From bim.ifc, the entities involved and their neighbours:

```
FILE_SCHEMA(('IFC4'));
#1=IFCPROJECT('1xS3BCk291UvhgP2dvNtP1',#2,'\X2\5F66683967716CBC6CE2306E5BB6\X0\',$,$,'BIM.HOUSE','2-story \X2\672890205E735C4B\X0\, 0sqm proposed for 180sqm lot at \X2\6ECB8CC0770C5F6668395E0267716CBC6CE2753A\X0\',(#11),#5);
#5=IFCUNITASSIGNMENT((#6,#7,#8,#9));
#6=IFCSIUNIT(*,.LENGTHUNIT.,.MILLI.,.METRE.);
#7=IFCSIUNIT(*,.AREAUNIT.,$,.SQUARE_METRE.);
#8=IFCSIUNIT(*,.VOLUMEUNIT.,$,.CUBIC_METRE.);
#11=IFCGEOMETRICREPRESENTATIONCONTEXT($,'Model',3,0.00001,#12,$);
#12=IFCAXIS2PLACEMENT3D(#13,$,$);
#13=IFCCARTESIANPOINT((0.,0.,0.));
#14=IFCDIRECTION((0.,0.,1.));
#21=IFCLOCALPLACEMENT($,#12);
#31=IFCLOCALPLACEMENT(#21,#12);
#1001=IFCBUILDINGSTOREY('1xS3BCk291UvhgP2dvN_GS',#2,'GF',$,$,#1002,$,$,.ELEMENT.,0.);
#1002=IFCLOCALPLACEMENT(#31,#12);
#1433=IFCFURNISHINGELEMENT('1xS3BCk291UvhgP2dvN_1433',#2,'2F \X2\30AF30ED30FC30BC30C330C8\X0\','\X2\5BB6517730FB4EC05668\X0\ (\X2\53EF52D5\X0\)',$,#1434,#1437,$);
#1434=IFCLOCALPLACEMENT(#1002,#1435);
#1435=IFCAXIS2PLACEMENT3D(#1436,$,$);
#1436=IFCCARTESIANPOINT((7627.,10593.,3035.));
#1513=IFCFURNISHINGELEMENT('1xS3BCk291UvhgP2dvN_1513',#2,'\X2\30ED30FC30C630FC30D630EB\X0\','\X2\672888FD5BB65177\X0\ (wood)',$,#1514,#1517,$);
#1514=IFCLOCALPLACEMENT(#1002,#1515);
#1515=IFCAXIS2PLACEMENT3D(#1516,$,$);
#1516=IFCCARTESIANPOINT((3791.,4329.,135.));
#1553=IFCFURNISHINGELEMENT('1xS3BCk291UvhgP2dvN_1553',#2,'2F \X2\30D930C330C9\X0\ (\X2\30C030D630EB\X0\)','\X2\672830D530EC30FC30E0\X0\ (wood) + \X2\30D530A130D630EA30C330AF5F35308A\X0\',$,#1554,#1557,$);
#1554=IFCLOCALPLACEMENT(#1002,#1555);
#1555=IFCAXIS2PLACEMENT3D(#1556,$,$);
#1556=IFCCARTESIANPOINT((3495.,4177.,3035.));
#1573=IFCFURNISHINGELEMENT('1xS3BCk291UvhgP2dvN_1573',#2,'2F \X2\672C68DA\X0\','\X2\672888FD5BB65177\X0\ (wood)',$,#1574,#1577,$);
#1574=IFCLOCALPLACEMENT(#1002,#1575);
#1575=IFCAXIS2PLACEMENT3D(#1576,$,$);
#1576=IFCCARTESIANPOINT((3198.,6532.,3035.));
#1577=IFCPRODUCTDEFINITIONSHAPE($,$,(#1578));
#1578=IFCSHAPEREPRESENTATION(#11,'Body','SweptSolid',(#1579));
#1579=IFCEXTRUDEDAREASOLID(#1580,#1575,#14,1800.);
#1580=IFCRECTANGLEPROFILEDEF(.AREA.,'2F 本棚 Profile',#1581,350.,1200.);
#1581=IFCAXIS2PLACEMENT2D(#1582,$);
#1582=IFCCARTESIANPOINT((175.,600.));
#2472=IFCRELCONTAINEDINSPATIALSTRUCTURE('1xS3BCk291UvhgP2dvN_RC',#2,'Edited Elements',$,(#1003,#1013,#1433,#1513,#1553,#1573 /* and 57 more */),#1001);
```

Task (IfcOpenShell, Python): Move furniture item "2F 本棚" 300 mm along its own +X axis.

```python
import ifcopenshell
import ifcopenshell.api.geometry
import ifcopenshell.util.placement

model = ifcopenshell.open("bim.ifc")

item = model.by_id(1573)
matrix = ifcopenshell.util.placement.get_local_placement(item.ObjectPlacement)
matrix[:3, 3] += matrix[:3, 0] * 300.0
ifcopenshell.api.geometry.edit_object_placement(model, product=item, matrix=matrix, is_si=False)

print(ifcopenshell.util.placement.get_local_placement(item.ObjectPlacement).round(3) + 0.0)

model.write("bim_updated.ifc")
```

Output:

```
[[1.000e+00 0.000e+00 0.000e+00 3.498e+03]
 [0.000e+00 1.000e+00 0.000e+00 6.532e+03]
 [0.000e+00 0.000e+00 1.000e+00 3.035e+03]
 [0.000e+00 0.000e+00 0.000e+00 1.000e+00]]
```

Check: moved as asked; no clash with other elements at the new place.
